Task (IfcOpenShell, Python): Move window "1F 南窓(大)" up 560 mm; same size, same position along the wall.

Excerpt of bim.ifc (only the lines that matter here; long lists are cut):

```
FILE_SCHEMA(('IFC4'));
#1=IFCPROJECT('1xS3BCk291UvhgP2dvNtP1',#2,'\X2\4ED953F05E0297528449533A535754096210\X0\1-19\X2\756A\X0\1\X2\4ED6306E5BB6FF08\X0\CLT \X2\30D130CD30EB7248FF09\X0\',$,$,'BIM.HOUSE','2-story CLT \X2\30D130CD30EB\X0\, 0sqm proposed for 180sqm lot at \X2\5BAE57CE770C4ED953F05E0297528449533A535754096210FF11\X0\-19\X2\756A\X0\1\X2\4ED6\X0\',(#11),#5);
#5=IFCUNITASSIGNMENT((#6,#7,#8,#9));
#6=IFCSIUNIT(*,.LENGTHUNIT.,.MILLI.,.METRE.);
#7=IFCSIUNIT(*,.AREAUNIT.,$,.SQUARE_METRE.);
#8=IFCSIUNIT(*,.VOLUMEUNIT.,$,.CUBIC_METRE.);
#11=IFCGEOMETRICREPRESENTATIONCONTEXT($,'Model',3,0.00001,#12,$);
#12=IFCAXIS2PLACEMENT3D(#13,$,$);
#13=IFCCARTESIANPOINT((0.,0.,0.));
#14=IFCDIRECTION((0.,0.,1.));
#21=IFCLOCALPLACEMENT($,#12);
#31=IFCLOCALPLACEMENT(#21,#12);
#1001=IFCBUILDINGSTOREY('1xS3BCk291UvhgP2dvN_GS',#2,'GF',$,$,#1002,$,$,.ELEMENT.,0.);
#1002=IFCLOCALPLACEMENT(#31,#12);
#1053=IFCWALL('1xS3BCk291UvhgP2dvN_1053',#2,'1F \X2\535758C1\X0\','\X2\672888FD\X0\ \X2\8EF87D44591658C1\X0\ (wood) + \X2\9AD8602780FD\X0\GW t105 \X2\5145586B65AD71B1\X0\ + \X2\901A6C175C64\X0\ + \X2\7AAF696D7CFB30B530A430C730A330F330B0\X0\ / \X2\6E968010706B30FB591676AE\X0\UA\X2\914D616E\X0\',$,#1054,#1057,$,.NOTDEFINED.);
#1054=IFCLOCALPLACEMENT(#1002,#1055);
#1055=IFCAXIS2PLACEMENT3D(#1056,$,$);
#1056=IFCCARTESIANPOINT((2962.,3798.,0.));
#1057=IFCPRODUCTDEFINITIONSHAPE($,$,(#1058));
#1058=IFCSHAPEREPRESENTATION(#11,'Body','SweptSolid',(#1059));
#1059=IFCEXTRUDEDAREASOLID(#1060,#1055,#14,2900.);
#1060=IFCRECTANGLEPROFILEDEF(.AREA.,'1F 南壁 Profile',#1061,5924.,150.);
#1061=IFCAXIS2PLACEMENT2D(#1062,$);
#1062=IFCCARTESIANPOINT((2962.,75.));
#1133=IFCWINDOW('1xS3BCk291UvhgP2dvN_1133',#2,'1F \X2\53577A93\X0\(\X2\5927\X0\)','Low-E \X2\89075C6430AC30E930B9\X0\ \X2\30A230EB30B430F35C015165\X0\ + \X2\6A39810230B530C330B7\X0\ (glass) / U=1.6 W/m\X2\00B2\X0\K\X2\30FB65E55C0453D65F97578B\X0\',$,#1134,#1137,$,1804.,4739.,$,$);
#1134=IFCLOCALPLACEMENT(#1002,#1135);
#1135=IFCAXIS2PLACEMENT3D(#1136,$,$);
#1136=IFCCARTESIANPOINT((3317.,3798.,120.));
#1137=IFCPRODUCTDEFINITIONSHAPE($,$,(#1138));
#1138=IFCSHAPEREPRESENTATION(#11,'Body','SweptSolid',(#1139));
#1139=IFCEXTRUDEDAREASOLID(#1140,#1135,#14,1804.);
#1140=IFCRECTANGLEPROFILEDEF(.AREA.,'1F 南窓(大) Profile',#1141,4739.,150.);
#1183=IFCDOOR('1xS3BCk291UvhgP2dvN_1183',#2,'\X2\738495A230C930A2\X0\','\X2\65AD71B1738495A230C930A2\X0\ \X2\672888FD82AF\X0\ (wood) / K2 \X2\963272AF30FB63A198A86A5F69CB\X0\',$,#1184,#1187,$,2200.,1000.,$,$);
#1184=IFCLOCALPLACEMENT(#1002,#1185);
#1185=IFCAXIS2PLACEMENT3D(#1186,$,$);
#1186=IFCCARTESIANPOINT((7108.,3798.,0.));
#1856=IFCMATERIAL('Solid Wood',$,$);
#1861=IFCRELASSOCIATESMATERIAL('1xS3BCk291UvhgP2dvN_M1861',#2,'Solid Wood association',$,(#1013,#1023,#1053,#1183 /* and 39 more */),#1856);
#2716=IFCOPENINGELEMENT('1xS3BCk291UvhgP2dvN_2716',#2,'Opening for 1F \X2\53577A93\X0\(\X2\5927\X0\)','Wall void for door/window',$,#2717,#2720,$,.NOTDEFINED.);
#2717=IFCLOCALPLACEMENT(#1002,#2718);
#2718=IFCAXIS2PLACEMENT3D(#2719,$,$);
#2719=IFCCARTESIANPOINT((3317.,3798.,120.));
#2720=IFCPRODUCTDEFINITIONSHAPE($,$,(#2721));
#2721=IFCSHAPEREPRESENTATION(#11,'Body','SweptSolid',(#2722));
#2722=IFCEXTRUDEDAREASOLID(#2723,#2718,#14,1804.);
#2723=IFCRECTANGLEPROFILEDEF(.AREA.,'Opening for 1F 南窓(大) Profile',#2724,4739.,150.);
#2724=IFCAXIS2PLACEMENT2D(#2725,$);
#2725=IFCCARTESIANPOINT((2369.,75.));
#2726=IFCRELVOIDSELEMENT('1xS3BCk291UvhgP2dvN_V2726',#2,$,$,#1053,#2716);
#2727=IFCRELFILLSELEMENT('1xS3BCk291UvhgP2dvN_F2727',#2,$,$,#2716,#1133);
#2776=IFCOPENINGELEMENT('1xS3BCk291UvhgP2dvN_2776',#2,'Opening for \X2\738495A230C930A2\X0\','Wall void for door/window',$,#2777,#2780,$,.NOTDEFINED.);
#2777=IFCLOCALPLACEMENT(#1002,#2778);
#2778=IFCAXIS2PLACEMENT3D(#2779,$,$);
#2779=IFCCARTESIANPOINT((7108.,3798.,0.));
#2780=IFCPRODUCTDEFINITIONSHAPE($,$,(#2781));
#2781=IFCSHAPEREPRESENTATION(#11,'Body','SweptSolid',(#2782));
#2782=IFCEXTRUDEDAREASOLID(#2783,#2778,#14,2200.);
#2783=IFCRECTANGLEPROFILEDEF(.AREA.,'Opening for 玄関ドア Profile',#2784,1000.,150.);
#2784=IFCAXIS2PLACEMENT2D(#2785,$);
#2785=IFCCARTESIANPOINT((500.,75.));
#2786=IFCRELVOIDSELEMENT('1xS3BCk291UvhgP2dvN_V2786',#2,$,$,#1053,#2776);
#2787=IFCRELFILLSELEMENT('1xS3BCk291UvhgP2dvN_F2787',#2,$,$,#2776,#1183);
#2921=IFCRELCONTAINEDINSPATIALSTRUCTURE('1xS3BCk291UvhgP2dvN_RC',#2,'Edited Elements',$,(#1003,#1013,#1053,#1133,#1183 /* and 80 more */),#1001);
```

```python
import numpy as np
import ifcopenshell
import ifcopenshell.api.geometry
import ifcopenshell.util.placement
import ifcopenshell.util.unit

model = ifcopenshell.open("bim.ifc")
unit_scale = ifcopenshell.util.unit.calculate_unit_scale(model)

window = model.by_guid("1xS3BCk291UvhgP2dvN_1133")
opening = window.FillsVoids[0].RelatingOpeningElement
dz = 0.56 / unit_scale

shift = np.array([0.0, 0.0, dz])
# The window is not placed relative to its opening, so move both.
for product in (opening, window):
    matrix = ifcopenshell.util.placement.get_local_placement(product.ObjectPlacement)
    matrix[:3, 3] += shift
    ifcopenshell.api.geometry.edit_object_placement(model, product=product, matrix=matrix, is_si=False)

print(f"moved by {dz * unit_scale:+.3f} m")

model.write("bim_edited.ifc")
```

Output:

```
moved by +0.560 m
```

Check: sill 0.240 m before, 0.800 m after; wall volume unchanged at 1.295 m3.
